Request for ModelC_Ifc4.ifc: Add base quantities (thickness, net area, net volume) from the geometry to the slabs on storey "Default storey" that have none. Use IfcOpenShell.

First a look at what the model holds.

```python
import ifcopenshell
import ifcopenshell.util.element
import ifcopenshell.util.unit

model = ifcopenshell.open("ModelC_Ifc4.ifc")
print(model.schema)
for unit_type in ("LENGTHUNIT", "AREAUNIT", "VOLUMEUNIT"):
    print(unit_type, ifcopenshell.util.unit.calculate_unit_scale(model, unit_type))
storey = next(s for s in model.by_type("IfcBuildingStorey") if s.Name == "Default storey")
slabs = [e for e in ifcopenshell.util.element.get_decomposition(storey) if e.is_a("IfcSlab")]
for e in sorted(slabs, key=lambda e: e.id()):
    print(e.id(), e.is_a(), e.Name, list(ifcopenshell.util.element.get_psets(e, qtos_only=True)), sep=" | ")
```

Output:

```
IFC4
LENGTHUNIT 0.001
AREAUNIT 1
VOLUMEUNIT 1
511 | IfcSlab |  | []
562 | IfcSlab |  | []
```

```python
import ifcopenshell
import ifcopenshell.api.pset
import ifcopenshell.geom
import ifcopenshell.util.element
import ifcopenshell.util.shape
import ifcopenshell.util.unit

model = ifcopenshell.open("ModelC_Ifc4.ifc")
unit_scale = ifcopenshell.util.unit.calculate_unit_scale(model)
area_scale = ifcopenshell.util.unit.calculate_unit_scale(model, "AREAUNIT")
volume_scale = ifcopenshell.util.unit.calculate_unit_scale(model, "VOLUMEUNIT")
settings = ifcopenshell.geom.settings()

storey = next(s for s in model.by_type("IfcBuildingStorey") if s.Name == "Default storey")
slabs = [e for e in ifcopenshell.util.element.get_decomposition(storey) if e.is_a("IfcSlab")]

for e in sorted(slabs, key=lambda e: e.id()):
    if ifcopenshell.util.element.get_psets(e, qtos_only=True, should_inherit=False):
        continue
    # Geometry comes back in metres, in the element's own axes.
    shape = ifcopenshell.geom.create_shape(settings, e)
    values = {
        "Width": ifcopenshell.util.shape.get_z(shape.geometry) / unit_scale,
        "NetArea": ifcopenshell.util.shape.get_footprint_area(shape.geometry) / area_scale,
        "NetVolume": ifcopenshell.util.shape.get_volume(shape.geometry) / volume_scale,
    }
    qto = ifcopenshell.api.pset.add_qto(model, product=e, name="Qto_SlabBaseQuantities")
    ifcopenshell.api.pset.edit_qto(model, qto=qto, properties=values)
    print(e.id(), {k: round(v, 3) for k, v in values.items()})

model.write("ModelC_Ifc4_v2.ifc")
```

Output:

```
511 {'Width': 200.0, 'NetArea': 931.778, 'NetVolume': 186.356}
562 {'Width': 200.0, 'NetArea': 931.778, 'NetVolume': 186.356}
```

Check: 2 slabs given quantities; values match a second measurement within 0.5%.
